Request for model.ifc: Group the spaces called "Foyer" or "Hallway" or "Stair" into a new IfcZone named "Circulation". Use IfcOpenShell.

First a look at what the model holds.

```python
import ifcopenshell

model = ifcopenshell.open("model.ifc")
print(model.schema)
seen = {}
for space in model.by_type("IfcSpace"):
    seen[space.LongName] = seen.get(space.LongName, 0) + 1
for name, count in sorted(seen.items(), key=str):
    print(count, "x", name)
print("zones:", [z.Name for z in model.by_type("IfcZone")][:20])
```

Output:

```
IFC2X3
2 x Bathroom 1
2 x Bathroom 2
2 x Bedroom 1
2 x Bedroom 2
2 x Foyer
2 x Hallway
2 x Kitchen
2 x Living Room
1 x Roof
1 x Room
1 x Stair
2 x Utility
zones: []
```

```python
import ifcopenshell
import ifcopenshell.api.group
import ifcopenshell.api.root

model = ifcopenshell.open("model.ifc")

names = {"Foyer", "Hallway", "Stair"}
spaces = [s for s in model.by_type("IfcSpace") if s.LongName in names]

zone = ifcopenshell.api.root.create_entity(model, ifc_class="IfcZone", name="Circulation")
ifcopenshell.api.group.assign_group(model, products=spaces, group=zone)
print(len(spaces), "spaces in", zone.Name)

model.write("model-out.ifc")
```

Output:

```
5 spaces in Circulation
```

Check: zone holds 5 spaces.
